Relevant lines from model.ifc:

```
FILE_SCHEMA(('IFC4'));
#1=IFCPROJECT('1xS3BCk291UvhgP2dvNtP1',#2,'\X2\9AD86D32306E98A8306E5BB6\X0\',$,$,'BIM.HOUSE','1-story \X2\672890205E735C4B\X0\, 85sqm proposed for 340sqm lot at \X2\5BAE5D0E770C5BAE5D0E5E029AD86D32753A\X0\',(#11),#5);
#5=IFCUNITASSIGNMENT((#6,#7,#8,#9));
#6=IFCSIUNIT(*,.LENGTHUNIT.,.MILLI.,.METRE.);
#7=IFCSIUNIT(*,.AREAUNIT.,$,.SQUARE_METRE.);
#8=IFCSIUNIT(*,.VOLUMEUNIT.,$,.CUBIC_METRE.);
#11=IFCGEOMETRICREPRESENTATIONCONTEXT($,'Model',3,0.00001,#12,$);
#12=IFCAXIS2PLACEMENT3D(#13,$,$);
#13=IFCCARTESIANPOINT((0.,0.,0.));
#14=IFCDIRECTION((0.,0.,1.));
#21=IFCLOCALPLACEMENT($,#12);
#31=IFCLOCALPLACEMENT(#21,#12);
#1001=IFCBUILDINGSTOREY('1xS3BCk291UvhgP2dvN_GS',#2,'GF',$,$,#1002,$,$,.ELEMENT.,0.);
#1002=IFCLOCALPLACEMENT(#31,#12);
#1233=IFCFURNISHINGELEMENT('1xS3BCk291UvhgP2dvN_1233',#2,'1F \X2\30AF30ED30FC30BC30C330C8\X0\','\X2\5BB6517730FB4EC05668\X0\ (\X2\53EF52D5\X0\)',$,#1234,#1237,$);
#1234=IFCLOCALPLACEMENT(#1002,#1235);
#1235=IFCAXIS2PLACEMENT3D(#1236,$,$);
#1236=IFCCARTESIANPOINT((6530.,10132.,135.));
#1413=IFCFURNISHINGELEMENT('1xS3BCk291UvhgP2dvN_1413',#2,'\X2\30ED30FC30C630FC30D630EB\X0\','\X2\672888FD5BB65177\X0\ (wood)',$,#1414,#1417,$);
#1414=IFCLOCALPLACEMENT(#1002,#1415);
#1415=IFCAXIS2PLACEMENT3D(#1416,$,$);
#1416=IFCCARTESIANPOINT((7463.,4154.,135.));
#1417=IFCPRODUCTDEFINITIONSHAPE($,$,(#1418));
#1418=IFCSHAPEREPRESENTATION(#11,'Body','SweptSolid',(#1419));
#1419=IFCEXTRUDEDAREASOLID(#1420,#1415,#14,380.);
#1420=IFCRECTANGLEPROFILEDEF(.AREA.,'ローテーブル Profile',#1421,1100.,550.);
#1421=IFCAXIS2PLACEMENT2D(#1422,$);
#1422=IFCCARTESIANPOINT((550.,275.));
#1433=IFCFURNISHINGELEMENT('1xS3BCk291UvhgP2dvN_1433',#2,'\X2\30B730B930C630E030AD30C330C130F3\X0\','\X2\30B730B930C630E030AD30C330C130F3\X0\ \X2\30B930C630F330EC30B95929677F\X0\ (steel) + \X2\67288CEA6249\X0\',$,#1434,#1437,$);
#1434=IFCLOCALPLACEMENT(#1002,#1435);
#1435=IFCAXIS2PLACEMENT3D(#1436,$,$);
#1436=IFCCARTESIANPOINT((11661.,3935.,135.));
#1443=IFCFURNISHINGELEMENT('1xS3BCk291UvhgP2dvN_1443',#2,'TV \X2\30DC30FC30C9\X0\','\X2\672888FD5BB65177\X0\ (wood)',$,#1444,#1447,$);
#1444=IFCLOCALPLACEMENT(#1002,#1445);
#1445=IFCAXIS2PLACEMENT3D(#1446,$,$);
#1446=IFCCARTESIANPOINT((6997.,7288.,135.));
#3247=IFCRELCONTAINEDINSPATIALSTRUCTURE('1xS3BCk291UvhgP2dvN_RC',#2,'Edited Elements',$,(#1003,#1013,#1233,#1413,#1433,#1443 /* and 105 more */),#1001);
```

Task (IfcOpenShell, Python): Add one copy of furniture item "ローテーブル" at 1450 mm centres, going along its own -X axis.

```python
import ifcopenshell
import ifcopenshell.api.geometry
import ifcopenshell.api.root
import ifcopenshell.util.element
import ifcopenshell.util.placement
import ifcopenshell.util.unit

model = ifcopenshell.open("model.ifc")
unit_scale = ifcopenshell.util.unit.calculate_unit_scale(model)


def reuse_history(source, copy):
    """copy_class also copies each property set's owner history, people and application; keep the originals."""
    for rel in copy.IsDefinedBy:
        if rel.is_a("IfcRelDefinesByProperties") and (history := rel.RelatingPropertyDefinition.OwnerHistory):
            rel.RelatingPropertyDefinition.OwnerHistory = source.OwnerHistory
            ifcopenshell.util.element.remove_deep2(model, history)


source = model.by_id(1413)
base = ifcopenshell.util.placement.get_local_placement(source.ObjectPlacement)
step = -base[:3, 0] * 1.45 / unit_scale

for i in range(1, 2):
    copy = ifcopenshell.api.root.copy_class(model, product=source)
    copy.Representation = ifcopenshell.util.element.copy_deep(
        model, source.Representation, exclude=["IfcGeometricRepresentationContext", "IfcRepresentationMap"]
    )
    reuse_history(source, copy)
    matrix = base.copy()
    matrix[:3, 3] += i * step
    print("added at", matrix[:3, 3].round(3) + 0.0)
    ifcopenshell.api.geometry.edit_object_placement(model, product=copy, matrix=matrix, is_si=False)

model.write("model_edited.ifc")
```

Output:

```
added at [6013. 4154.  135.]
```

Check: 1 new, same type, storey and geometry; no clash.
